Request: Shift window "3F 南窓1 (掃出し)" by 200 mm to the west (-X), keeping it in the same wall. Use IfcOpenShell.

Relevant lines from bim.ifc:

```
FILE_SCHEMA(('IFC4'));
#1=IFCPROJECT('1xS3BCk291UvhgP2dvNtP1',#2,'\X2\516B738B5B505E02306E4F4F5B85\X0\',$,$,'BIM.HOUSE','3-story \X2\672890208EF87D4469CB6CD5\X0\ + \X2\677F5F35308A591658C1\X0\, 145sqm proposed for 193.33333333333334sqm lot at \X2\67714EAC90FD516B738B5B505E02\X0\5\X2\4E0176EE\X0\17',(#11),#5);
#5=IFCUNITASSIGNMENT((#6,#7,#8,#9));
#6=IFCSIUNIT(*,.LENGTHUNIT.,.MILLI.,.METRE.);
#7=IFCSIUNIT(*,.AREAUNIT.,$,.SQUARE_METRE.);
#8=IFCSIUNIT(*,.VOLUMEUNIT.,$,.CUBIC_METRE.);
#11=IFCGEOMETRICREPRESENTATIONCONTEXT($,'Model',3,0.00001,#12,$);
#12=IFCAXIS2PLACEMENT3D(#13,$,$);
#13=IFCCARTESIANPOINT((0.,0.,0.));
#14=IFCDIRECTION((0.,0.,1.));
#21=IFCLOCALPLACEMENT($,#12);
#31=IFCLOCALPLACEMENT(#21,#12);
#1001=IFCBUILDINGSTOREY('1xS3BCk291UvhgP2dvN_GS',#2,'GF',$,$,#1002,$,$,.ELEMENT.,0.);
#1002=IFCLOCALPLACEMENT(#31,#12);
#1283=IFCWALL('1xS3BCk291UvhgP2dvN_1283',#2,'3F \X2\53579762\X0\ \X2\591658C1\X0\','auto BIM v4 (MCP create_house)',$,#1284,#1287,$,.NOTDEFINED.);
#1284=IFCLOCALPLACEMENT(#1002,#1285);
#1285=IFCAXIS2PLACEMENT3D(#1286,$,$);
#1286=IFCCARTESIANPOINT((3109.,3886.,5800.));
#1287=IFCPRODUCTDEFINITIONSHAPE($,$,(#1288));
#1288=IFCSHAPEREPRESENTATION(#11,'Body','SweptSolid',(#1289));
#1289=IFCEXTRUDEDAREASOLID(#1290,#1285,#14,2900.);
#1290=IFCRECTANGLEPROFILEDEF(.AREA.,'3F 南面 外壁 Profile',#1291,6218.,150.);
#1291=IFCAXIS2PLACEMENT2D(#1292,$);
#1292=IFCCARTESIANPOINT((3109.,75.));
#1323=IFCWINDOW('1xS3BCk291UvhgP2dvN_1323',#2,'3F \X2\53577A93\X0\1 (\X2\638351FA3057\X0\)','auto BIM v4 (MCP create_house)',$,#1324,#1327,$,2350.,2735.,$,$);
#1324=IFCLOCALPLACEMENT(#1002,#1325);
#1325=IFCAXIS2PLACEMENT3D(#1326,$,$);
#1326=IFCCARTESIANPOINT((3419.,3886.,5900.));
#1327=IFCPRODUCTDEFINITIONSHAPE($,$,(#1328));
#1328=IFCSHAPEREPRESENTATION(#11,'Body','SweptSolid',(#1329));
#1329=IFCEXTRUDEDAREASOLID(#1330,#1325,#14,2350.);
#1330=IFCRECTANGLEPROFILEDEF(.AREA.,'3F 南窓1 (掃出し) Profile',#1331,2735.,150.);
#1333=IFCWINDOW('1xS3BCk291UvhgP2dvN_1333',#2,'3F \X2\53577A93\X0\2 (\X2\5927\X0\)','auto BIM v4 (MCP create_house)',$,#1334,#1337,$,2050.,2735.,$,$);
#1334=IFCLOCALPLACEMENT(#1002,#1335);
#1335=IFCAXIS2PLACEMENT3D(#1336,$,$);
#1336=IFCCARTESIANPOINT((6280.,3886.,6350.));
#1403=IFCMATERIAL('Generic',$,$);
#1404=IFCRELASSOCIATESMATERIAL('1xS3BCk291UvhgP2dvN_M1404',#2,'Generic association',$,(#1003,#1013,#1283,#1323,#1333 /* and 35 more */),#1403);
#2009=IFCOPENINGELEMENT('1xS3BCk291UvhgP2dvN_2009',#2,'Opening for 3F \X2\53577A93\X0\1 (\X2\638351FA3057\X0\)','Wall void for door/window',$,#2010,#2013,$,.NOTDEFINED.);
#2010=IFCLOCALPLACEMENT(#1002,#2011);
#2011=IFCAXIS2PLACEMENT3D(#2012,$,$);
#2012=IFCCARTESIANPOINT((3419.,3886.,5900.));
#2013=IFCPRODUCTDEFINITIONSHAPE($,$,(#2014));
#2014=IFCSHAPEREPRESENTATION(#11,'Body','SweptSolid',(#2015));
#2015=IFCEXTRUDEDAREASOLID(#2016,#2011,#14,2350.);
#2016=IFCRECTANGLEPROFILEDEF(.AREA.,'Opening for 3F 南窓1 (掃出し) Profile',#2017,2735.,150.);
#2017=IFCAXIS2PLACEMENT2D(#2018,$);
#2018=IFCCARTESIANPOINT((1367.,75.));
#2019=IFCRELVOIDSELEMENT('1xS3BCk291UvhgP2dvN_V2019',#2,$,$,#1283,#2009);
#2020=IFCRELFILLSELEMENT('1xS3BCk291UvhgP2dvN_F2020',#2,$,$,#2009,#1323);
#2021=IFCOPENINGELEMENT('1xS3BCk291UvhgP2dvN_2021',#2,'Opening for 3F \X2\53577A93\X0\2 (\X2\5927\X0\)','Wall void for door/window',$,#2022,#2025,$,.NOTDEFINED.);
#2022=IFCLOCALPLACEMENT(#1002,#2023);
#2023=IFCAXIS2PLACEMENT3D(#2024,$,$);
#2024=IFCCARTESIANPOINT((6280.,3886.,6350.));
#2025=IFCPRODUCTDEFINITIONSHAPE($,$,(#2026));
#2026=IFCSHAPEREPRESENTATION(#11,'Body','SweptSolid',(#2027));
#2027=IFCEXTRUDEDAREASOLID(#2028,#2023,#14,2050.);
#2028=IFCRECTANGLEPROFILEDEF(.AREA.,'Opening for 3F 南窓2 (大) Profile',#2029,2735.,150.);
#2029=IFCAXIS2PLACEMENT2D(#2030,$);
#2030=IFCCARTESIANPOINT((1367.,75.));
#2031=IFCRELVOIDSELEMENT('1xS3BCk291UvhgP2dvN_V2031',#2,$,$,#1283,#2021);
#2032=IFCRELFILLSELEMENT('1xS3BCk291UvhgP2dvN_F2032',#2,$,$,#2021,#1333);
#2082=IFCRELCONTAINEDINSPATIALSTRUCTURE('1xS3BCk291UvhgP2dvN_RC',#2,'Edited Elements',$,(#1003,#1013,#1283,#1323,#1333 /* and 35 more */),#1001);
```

```python
import ifcopenshell
import ifcopenshell.api.geometry
import ifcopenshell.util.placement
import ifcopenshell.util.unit

model = ifcopenshell.open("bim.ifc")
unit_scale = ifcopenshell.util.unit.calculate_unit_scale(model)

window = model.by_guid("1xS3BCk291UvhgP2dvN_1323")
opening = window.FillsVoids[0].RelatingOpeningElement
wall = opening.VoidsElements[0].RelatingBuildingElement

wall_matrix = ifcopenshell.util.placement.get_local_placement(wall.ObjectPlacement)
shift = wall_matrix[:3, 0] * -0.2 / unit_scale
before = ifcopenshell.util.placement.get_local_placement(window.ObjectPlacement)[:3, 3].copy()

# The window is not placed relative to its opening, so move both.
for product in (opening, window):
    matrix = ifcopenshell.util.placement.get_local_placement(product.ObjectPlacement)
    matrix[:3, 3] += shift
    ifcopenshell.api.geometry.edit_object_placement(model, product=product, matrix=matrix, is_si=False)

after = ifcopenshell.util.placement.get_local_placement(window.ObjectPlacement)[:3, 3]
print("window moved by", (after - before).round(3) + 0.0)

model.write("bim_edited.ifc")
```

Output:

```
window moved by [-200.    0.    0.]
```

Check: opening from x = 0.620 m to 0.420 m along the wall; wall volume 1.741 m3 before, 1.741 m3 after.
